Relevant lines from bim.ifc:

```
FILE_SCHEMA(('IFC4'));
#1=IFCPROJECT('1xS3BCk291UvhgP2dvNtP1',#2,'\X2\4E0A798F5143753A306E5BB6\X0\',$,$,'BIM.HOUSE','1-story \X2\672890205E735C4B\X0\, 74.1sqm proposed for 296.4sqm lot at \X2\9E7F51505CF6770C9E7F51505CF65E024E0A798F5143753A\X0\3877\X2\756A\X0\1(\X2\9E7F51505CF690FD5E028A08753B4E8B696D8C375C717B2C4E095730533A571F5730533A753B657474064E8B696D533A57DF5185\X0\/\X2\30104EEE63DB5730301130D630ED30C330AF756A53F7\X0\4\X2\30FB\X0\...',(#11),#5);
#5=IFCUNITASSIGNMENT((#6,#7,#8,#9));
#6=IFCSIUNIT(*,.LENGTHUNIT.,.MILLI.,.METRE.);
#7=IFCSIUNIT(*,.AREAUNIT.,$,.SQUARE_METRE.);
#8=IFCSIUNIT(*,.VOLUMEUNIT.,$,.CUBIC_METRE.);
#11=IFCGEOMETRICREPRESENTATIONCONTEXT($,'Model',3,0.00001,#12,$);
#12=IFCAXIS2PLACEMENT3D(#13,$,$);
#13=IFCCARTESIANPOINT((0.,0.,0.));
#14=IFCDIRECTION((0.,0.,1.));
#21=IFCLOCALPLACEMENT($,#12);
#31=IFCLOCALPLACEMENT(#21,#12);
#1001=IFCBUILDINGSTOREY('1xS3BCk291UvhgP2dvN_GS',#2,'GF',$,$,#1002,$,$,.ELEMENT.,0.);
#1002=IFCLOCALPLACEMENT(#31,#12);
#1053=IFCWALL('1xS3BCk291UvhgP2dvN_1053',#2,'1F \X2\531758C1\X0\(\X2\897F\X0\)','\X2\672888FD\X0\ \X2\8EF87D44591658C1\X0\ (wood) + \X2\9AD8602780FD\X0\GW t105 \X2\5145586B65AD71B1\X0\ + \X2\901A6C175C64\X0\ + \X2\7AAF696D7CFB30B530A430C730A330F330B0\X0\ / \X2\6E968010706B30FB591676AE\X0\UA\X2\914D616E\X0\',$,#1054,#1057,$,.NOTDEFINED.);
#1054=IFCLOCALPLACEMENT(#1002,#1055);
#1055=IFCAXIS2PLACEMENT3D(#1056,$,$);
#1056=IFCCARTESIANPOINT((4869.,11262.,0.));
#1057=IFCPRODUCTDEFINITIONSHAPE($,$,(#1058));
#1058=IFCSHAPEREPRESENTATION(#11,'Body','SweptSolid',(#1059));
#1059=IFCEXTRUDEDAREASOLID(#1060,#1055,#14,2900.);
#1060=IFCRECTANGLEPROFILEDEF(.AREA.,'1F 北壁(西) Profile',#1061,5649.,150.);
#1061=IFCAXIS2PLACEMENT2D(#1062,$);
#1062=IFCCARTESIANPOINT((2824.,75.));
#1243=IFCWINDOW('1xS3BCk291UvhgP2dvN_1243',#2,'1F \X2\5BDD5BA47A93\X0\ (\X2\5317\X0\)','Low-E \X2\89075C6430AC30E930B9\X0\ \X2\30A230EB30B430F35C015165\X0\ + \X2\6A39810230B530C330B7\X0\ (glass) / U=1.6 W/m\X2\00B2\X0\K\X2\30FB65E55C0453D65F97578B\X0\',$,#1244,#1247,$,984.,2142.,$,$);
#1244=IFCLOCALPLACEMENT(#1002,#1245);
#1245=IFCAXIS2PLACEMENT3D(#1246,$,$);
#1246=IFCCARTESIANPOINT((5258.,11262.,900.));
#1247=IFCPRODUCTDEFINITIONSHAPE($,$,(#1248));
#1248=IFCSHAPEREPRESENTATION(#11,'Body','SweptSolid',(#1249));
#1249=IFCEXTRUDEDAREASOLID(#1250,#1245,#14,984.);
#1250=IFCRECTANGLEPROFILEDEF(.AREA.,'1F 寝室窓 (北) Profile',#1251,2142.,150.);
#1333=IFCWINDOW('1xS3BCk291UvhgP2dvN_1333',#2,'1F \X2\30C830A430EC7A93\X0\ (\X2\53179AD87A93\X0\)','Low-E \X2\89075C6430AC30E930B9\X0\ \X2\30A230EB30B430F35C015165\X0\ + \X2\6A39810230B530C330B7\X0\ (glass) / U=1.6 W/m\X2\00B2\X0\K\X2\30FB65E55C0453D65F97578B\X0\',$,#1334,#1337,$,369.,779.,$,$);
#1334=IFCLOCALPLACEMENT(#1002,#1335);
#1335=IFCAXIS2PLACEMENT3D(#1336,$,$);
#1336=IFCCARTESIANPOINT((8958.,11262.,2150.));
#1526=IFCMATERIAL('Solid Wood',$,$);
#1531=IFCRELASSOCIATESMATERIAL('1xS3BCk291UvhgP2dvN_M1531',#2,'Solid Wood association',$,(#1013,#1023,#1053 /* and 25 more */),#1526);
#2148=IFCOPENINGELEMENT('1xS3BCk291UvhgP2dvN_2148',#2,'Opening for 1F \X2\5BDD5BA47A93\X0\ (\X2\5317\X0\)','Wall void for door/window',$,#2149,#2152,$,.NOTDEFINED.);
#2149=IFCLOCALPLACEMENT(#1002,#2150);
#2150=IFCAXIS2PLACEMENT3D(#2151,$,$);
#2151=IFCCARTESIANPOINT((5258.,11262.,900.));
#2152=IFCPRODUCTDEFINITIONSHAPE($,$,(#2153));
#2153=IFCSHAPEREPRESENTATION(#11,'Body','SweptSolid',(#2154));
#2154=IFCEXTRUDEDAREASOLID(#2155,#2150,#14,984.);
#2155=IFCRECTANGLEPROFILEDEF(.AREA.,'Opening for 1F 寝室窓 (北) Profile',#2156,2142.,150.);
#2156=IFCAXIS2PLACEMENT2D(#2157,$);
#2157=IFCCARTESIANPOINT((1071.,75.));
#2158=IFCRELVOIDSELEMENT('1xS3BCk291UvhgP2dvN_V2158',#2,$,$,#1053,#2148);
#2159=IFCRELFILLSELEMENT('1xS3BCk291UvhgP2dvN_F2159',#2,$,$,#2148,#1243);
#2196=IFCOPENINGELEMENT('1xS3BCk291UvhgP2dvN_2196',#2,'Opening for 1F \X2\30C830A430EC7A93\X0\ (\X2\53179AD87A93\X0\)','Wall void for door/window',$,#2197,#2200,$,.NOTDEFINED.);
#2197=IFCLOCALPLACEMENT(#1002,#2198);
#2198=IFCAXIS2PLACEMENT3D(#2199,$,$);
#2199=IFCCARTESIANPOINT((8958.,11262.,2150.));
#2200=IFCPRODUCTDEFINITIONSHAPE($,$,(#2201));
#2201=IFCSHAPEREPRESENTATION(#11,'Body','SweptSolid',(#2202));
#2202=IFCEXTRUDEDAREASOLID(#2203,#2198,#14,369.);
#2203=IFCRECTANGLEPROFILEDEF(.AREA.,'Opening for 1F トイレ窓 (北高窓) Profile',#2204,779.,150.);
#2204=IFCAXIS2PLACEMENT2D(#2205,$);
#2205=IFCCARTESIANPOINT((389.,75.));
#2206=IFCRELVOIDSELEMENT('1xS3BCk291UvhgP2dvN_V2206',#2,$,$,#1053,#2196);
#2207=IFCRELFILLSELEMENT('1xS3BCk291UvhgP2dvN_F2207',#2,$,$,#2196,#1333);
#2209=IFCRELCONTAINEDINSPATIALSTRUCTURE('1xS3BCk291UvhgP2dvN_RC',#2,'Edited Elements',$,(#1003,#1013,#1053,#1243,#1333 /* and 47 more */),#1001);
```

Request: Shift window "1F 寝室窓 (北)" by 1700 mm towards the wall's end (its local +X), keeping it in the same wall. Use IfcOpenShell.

```python
import ifcopenshell
import ifcopenshell.api.geometry
import ifcopenshell.util.placement

model = ifcopenshell.open("bim.ifc")

window = model.by_id(1243)
opening = window.FillsVoids[0].RelatingOpeningElement
wall = opening.VoidsElements[0].RelatingBuildingElement

wall_matrix = ifcopenshell.util.placement.get_local_placement(wall.ObjectPlacement)
shift = wall_matrix[:3, 0] * 1700.0
before = ifcopenshell.util.placement.get_local_placement(window.ObjectPlacement)[:3, 3].copy()

# The window is not placed relative to its opening, so move both.
for product in (opening, window):
    matrix = ifcopenshell.util.placement.get_local_placement(product.ObjectPlacement)
    matrix[:3, 3] += shift
    ifcopenshell.api.geometry.edit_object_placement(model, product=product, matrix=matrix, is_si=False)

after = ifcopenshell.util.placement.get_local_placement(window.ObjectPlacement)[:3, 3]
print("window moved by", (after - before).round(3) + 0.0)

model.write("bim_v2.ifc")
```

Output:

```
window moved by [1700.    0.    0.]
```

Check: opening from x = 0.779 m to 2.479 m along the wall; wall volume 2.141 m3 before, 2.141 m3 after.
